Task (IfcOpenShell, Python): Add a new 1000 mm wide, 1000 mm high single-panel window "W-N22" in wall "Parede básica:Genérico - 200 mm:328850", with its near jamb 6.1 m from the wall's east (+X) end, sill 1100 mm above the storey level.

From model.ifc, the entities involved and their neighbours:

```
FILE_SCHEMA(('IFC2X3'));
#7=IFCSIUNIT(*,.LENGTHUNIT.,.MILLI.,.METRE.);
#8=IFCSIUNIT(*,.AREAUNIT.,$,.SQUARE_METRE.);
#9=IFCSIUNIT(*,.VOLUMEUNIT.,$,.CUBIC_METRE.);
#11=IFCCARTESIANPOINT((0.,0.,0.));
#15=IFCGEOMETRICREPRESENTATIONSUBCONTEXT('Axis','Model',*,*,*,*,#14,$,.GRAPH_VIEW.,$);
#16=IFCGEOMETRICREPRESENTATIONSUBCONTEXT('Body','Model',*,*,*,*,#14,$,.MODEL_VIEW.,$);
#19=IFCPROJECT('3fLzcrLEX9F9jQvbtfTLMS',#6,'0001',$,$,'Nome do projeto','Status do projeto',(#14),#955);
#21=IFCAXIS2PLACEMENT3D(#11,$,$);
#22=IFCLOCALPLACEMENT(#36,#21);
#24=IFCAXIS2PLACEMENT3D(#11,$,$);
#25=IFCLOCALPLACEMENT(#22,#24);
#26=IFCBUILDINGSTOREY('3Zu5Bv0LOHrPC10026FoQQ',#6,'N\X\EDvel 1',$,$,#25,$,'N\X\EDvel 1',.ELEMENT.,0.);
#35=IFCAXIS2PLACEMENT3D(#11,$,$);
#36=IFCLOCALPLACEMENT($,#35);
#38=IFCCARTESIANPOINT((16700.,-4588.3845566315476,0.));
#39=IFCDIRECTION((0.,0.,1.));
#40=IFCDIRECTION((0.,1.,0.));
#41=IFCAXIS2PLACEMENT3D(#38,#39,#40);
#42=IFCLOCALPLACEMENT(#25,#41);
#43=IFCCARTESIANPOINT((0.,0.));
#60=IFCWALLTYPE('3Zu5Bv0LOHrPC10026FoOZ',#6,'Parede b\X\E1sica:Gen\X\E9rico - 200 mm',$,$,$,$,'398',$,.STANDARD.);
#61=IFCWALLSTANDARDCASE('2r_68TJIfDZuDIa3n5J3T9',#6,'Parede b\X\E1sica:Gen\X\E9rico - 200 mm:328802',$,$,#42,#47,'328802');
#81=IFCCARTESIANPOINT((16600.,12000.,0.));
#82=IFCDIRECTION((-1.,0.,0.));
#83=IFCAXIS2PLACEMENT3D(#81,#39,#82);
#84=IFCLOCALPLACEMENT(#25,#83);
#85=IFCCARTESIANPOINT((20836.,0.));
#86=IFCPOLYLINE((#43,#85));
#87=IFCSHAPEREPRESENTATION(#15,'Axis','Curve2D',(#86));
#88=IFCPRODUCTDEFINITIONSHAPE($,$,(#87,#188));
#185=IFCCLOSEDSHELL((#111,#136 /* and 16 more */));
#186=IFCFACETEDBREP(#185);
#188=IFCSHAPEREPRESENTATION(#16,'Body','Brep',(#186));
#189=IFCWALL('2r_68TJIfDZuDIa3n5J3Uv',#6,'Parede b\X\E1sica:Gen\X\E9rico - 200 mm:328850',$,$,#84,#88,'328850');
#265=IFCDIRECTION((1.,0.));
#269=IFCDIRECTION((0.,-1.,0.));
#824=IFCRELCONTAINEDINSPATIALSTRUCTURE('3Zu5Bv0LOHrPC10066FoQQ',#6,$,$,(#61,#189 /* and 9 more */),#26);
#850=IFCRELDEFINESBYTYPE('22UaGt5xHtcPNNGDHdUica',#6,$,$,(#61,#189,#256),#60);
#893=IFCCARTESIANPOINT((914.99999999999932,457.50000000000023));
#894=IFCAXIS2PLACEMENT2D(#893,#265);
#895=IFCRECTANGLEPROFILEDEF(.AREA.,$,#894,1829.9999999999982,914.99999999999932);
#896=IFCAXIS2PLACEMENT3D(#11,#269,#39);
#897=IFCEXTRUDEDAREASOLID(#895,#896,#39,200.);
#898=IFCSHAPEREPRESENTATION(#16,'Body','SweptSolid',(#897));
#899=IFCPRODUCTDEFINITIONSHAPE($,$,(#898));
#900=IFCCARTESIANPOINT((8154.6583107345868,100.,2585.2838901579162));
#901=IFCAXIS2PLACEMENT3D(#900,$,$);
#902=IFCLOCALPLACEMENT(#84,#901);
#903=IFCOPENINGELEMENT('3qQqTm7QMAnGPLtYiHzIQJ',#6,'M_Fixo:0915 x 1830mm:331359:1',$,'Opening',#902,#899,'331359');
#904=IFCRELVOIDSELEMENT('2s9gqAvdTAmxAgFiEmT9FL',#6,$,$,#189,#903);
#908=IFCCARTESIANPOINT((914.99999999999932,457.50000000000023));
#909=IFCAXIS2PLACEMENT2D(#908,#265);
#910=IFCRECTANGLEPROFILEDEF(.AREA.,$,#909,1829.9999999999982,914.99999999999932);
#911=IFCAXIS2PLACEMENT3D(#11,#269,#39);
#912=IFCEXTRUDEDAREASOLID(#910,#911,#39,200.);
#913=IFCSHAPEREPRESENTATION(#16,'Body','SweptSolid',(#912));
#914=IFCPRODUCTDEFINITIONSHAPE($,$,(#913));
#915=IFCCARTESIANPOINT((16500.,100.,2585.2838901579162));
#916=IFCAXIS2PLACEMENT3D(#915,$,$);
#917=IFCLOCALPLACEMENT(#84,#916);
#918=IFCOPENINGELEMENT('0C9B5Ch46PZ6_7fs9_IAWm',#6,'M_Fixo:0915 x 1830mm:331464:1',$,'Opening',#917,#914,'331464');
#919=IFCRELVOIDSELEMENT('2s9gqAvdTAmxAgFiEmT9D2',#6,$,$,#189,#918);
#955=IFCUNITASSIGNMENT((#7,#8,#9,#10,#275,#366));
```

```python
import numpy as np
import ifcopenshell
import ifcopenshell.api.feature
import ifcopenshell.api.geometry
import ifcopenshell.api.root
import ifcopenshell.api.spatial
import ifcopenshell.api.type
import ifcopenshell.geom
import ifcopenshell.util.element
import ifcopenshell.util.placement
import ifcopenshell.util.representation
import ifcopenshell.util.shape
import ifcopenshell.util.unit

model = ifcopenshell.open("model.ifc")
unit_scale = ifcopenshell.util.unit.calculate_unit_scale(model)
settings = ifcopenshell.geom.settings()


def volume(element):
    """Net volume in cubic metres, openings subtracted."""
    shape = ifcopenshell.geom.create_shape(settings, element)
    return ifcopenshell.util.shape.get_volume(shape.geometry)


wall = model.by_id(189)
storey = ifcopenshell.util.element.get_container(wall, ifc_class="IfcBuildingStorey")
context = ifcopenshell.util.representation.get_context(model, "Model", "Body", "MODEL_VIEW")
before = volume(wall)

width, height, from_end, sill = 1, 1, 6.1, 1.1  # metres

# The wall runs along its own X axis, and the end named is its -X end.
wall_shape = ifcopenshell.geom.create_shape(settings, wall)
x, y, z = ifcopenshell.util.shape.get_vertices(wall_shape.geometry).T
start = x.min() + from_end
face, thickness = float(y.min()), float(y.max() - y.min())
wall_matrix = ifcopenshell.util.placement.get_local_placement(wall.ObjectPlacement)
level = ifcopenshell.util.placement.get_local_placement(storey.ObjectPlacement)[2, 3]


def in_wall(x, y):
    """Placement at x, y metres in the wall's axes, at sill height."""
    matrix = wall_matrix.copy()
    matrix[:, 3] = wall_matrix @ np.array([x / unit_scale, y / unit_scale, 0.0, 1.0])
    matrix[2, 3] = level + sill / unit_scale
    return matrix


# Opening: a box that overshoots both wall faces by 50 mm.
opening = ifcopenshell.api.root.create_entity(model, ifc_class="IfcOpeningElement")
box = ifcopenshell.api.geometry.add_wall_representation(
    model, context=context, length=width, height=height, thickness=thickness + 0.1
)
ifcopenshell.api.geometry.assign_representation(model, product=opening, representation=box)
ifcopenshell.api.geometry.edit_object_placement(model, product=opening, matrix=in_wall(start, face - 0.05), is_si=False)
ifcopenshell.api.feature.add_feature(model, feature=opening, element=wall)

window = ifcopenshell.api.root.create_entity(model, ifc_class="IfcWindow", name="W-N22")
window.OverallWidth, window.OverallHeight = width / unit_scale, height / unit_scale
body = ifcopenshell.api.geometry.add_window_representation(
    model,
    context=context,
    overall_width=window.OverallWidth,
    overall_height=window.OverallHeight,
    partition_type="SINGLE_PANEL",
)
ifcopenshell.api.geometry.assign_representation(model, product=window, representation=body)
ifcopenshell.api.spatial.assign_container(model, products=[window], relating_structure=storey)
fills = ifcopenshell.api.feature.add_filling(model, opening=opening, element=window)
fills.OwnerHistory = window.OwnerHistory  # required in IFC2X3

# IFC2X3 keeps the operation on the window style.
style = ifcopenshell.api.root.create_entity(model, ifc_class="IfcWindowStyle", name="W-N22")
style.OperationType, style.ConstructionType = "SINGLE_PANEL", "NOTDEFINED"
style.ParameterTakesPrecedence = style.Sizeable = False
ifcopenshell.api.type.assign_type(model, related_objects=[window], relating_type=style)

# Centre the window in the wall's thickness.
ifcopenshell.api.geometry.edit_object_placement(model, product=window, matrix=in_wall(start, face), is_si=False)
window_shape = ifcopenshell.geom.create_shape(settings, window)
depth = ifcopenshell.util.shape.get_vertices(window_shape.geometry)[:, 1]
offset = face + thickness / 2 - (depth.min() + depth.max()) / 2
ifcopenshell.api.geometry.edit_object_placement(model, product=window, matrix=in_wall(start, offset), is_si=False)

after = volume(wall)

print(f"wall volume {before:.3f} -> {after:.3f} m3")

model.write("model_v2.ifc")
```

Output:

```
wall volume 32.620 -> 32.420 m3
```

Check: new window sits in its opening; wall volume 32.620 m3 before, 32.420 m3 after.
